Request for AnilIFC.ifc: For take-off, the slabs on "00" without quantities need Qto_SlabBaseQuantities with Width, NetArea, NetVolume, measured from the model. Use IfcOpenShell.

First a look at what the model holds.

```python
import ifcopenshell
import ifcopenshell.util.element
import ifcopenshell.util.unit

model = ifcopenshell.open("AnilIFC.ifc")
print(model.schema)
for unit_type in ("LENGTHUNIT", "AREAUNIT", "VOLUMEUNIT"):
    print(unit_type, ifcopenshell.util.unit.calculate_unit_scale(model, unit_type))
storey = next(s for s in model.by_type("IfcBuildingStorey") if s.Name == "00")
slabs = [e for e in ifcopenshell.util.element.get_decomposition(storey) if e.is_a("IfcSlab")]
for e in sorted(slabs, key=lambda e: e.id()):
    print(e.id(), e.is_a(), e.Name, list(ifcopenshell.util.element.get_psets(e, qtos_only=True)), sep=" | ")
```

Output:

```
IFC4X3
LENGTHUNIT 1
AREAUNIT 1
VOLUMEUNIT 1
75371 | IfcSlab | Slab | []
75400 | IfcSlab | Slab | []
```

```python
import ifcopenshell
import ifcopenshell.api.pset
import ifcopenshell.geom
import ifcopenshell.util.element
import ifcopenshell.util.shape
import ifcopenshell.util.unit

model = ifcopenshell.open("AnilIFC.ifc")
unit_scale = ifcopenshell.util.unit.calculate_unit_scale(model)
area_scale = ifcopenshell.util.unit.calculate_unit_scale(model, "AREAUNIT")
volume_scale = ifcopenshell.util.unit.calculate_unit_scale(model, "VOLUMEUNIT")
settings = ifcopenshell.geom.settings()

storey = next(s for s in model.by_type("IfcBuildingStorey") if s.Name == "00")
slabs = [e for e in ifcopenshell.util.element.get_decomposition(storey) if e.is_a("IfcSlab")]

for e in sorted(slabs, key=lambda e: e.id()):
    if ifcopenshell.util.element.get_psets(e, qtos_only=True, should_inherit=False):
        continue
    # Geometry comes back in metres, in the element's own axes.
    shape = ifcopenshell.geom.create_shape(settings, e)
    values = {
        "Width": ifcopenshell.util.shape.get_z(shape.geometry) / unit_scale,
        "NetArea": ifcopenshell.util.shape.get_footprint_area(shape.geometry) / area_scale,
        "NetVolume": ifcopenshell.util.shape.get_volume(shape.geometry) / volume_scale,
    }
    qto = ifcopenshell.api.pset.add_qto(model, product=e, name="Qto_SlabBaseQuantities")
    ifcopenshell.api.pset.edit_qto(model, qto=qto, properties=values)
    print(e.id(), {k: round(v, 3) for k, v in values.items()})

model.write("AnilIFC_edited.ifc")
```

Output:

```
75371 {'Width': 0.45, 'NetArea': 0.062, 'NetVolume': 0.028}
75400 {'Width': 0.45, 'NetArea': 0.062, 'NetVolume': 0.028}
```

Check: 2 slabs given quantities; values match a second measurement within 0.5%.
